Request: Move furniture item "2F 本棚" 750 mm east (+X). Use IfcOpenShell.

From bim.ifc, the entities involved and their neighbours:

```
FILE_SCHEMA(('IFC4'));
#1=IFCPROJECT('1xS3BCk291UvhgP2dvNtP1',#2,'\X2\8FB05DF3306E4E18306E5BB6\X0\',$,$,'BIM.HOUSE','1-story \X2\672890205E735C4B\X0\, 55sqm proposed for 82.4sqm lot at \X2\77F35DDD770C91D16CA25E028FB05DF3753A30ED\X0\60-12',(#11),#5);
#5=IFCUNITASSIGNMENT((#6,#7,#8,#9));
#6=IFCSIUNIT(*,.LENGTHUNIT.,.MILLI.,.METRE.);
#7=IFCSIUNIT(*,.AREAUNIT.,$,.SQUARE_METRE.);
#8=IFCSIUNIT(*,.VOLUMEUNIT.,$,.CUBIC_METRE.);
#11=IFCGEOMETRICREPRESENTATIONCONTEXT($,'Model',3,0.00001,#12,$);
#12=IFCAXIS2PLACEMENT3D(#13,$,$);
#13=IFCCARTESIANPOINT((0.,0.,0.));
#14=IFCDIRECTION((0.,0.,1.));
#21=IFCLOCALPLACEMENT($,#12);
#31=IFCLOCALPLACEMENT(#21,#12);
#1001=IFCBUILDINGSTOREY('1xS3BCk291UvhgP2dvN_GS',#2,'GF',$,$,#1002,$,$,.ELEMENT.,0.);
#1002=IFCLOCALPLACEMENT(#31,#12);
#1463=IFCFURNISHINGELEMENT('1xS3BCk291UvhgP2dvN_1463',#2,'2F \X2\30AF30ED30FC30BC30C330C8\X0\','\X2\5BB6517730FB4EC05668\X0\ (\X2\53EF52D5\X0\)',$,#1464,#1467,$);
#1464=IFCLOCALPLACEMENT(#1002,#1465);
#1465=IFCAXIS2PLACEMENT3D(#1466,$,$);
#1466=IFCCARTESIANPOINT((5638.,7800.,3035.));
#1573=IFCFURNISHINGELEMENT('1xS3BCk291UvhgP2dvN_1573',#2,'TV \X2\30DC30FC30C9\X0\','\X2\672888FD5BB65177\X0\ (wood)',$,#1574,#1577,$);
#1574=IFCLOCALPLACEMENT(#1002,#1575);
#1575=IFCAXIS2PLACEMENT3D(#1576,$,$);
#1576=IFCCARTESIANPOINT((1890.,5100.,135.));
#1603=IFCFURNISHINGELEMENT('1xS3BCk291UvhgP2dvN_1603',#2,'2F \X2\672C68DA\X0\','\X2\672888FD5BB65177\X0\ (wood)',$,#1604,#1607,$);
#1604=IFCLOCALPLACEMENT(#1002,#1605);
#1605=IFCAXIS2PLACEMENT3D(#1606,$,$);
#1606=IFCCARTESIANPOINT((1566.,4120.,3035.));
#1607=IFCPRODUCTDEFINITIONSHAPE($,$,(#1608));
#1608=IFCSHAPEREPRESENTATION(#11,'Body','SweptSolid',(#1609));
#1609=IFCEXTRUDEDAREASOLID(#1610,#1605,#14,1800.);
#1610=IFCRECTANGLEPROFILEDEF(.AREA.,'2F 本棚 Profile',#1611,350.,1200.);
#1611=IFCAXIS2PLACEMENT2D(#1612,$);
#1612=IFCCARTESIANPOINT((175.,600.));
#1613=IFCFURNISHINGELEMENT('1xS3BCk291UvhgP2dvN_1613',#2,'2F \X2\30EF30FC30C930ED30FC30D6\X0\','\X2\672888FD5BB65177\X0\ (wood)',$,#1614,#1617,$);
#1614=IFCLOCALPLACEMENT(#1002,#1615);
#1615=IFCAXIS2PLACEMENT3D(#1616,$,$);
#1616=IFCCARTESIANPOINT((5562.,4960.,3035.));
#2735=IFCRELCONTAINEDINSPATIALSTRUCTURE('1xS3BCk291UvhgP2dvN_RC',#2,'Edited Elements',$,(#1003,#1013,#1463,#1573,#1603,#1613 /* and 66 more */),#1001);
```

```python
import ifcopenshell
import ifcopenshell.api.geometry
import ifcopenshell.util.placement
import ifcopenshell.util.unit

model = ifcopenshell.open("bim.ifc")
unit_scale = ifcopenshell.util.unit.calculate_unit_scale(model)

item = model.by_id(1603)
matrix = ifcopenshell.util.placement.get_local_placement(item.ObjectPlacement)
matrix[0, 3] += 0.75 / unit_scale
ifcopenshell.api.geometry.edit_object_placement(model, product=item, matrix=matrix, is_si=False)

print(ifcopenshell.util.placement.get_local_placement(item.ObjectPlacement).round(3) + 0.0)

model.write("bim_v2.ifc")
```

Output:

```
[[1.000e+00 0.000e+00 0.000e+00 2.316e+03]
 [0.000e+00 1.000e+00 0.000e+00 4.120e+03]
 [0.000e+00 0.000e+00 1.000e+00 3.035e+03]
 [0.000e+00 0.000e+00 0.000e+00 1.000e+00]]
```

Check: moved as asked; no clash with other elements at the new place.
